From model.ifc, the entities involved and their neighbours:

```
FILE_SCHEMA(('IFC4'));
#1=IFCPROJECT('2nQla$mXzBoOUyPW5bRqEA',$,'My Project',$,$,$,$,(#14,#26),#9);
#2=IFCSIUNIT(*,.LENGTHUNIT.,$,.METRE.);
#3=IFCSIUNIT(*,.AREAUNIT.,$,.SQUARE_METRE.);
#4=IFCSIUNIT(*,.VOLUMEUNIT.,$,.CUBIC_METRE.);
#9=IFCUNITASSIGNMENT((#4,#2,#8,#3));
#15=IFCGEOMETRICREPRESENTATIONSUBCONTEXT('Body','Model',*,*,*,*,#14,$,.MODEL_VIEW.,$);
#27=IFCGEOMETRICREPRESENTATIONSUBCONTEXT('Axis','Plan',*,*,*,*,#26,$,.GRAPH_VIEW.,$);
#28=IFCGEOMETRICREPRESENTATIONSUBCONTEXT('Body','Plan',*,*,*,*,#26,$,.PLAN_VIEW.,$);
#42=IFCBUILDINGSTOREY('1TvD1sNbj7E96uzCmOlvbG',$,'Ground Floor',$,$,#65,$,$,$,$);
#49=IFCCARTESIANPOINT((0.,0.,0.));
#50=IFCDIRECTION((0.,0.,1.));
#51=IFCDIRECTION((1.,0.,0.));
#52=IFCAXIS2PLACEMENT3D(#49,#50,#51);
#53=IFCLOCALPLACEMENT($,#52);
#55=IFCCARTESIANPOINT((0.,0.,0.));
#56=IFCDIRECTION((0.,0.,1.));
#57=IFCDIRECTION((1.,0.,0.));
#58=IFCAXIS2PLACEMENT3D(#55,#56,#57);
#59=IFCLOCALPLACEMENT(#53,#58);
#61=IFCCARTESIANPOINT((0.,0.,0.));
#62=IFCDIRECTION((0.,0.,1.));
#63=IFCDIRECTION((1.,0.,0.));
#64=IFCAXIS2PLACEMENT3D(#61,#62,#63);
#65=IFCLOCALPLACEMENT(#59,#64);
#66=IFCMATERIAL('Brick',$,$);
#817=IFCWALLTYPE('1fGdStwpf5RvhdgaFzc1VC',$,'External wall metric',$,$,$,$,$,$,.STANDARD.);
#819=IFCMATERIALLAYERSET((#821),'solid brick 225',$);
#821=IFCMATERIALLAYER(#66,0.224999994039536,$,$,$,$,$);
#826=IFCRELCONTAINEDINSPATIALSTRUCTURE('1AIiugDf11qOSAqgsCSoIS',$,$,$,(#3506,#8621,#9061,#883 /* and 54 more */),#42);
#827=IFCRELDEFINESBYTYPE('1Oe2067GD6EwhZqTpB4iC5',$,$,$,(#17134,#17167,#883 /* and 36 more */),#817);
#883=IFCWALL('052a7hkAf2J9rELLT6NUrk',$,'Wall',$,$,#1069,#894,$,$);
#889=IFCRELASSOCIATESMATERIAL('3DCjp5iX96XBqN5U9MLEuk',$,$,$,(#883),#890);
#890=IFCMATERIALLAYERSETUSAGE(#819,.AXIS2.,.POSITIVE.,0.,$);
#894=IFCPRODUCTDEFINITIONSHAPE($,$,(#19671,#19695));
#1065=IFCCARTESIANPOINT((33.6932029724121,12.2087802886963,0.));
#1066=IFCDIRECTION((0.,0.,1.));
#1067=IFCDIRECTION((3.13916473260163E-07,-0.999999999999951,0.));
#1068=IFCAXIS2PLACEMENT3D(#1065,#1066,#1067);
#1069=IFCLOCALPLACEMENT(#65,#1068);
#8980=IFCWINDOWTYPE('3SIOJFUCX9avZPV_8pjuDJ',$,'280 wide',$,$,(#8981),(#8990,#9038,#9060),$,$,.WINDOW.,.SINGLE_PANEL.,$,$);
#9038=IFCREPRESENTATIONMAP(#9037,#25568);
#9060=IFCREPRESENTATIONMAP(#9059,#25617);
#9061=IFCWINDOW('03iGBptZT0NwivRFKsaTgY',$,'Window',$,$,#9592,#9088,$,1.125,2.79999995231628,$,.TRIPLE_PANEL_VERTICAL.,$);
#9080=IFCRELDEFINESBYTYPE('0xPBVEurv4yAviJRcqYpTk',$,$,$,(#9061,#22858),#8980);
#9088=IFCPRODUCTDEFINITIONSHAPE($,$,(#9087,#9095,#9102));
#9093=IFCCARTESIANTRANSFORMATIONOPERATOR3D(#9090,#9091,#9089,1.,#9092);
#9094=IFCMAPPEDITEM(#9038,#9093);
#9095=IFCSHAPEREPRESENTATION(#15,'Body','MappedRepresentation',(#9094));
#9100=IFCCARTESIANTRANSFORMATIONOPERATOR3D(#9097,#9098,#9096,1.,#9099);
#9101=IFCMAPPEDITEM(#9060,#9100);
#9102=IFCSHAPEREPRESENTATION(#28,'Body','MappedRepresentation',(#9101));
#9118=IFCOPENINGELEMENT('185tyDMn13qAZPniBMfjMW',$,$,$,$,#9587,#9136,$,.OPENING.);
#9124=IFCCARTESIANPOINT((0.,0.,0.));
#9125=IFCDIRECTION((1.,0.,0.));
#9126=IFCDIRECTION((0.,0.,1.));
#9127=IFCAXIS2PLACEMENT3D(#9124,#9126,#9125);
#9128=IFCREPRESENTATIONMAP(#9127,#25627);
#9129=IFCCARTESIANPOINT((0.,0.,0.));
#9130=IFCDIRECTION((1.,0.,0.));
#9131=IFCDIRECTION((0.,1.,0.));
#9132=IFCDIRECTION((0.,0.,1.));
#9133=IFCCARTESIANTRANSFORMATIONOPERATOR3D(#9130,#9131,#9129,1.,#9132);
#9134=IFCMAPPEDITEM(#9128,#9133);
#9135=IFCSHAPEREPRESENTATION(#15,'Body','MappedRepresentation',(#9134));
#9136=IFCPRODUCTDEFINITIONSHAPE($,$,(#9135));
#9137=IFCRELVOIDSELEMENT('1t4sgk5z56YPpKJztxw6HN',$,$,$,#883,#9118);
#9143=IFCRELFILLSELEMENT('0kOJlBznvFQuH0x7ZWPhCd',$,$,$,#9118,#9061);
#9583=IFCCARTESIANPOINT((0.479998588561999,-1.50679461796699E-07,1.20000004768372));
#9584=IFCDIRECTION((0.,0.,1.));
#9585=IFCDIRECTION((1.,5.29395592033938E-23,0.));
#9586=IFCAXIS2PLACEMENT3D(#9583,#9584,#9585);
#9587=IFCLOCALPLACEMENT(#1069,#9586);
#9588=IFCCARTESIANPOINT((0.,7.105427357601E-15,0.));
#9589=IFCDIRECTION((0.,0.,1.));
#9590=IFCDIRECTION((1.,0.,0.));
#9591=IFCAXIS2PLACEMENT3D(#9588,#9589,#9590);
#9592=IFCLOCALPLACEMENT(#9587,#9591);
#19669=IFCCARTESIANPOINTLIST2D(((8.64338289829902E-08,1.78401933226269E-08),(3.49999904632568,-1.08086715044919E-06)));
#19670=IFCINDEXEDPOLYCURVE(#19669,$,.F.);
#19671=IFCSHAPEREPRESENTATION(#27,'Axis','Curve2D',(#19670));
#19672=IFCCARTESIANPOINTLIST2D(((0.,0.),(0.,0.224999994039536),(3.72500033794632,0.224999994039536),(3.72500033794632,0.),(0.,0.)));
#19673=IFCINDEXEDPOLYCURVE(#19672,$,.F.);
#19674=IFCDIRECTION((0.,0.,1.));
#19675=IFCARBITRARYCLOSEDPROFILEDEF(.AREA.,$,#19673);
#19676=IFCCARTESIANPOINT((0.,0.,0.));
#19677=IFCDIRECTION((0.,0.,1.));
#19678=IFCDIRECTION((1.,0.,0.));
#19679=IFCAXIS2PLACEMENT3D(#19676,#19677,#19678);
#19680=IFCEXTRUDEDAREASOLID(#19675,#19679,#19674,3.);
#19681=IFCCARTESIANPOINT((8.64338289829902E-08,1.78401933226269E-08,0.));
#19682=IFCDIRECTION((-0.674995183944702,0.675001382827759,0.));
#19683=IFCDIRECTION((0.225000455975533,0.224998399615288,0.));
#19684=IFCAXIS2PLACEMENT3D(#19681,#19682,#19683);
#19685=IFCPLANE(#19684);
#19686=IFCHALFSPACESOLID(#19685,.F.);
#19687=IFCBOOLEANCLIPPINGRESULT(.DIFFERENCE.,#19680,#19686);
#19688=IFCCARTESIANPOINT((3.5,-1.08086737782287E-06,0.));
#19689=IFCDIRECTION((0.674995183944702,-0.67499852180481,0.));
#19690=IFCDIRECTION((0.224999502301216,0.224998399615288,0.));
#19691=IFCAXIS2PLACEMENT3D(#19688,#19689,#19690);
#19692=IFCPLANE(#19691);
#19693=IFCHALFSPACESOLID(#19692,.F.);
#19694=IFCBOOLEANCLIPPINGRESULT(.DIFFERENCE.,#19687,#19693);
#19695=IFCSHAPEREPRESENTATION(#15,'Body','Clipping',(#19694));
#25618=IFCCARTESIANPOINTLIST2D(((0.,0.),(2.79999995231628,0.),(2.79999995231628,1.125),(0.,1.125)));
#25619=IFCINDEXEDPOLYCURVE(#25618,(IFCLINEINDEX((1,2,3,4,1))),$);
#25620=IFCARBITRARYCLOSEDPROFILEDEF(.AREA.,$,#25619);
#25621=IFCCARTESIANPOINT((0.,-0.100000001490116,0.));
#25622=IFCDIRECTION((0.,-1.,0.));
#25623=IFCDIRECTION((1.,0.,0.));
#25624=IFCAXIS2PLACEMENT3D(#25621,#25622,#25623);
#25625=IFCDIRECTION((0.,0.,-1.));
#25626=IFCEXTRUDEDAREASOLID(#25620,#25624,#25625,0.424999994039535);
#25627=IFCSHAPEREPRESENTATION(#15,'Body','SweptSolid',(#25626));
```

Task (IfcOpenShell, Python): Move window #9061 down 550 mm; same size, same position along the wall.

```python
import numpy as np
import ifcopenshell
import ifcopenshell.api.geometry
import ifcopenshell.util.placement
import ifcopenshell.util.unit

model = ifcopenshell.open("model.ifc")
unit_scale = ifcopenshell.util.unit.calculate_unit_scale(model)

window = model.by_guid("03iGBptZT0NwivRFKsaTgY")
opening = window.FillsVoids[0].RelatingOpeningElement
dz = -0.55 / unit_scale

shift = np.array([0.0, 0.0, dz])
# The window is placed relative to its opening, so it follows when the opening moves.
matrix = ifcopenshell.util.placement.get_local_placement(opening.ObjectPlacement)
matrix[:3, 3] += shift
ifcopenshell.api.geometry.edit_object_placement(
    model, product=opening, matrix=matrix, is_si=False, should_transform_children=True
)

print(f"moved by {dz * unit_scale:+.3f} m")

model.write("model_edited.ifc")
```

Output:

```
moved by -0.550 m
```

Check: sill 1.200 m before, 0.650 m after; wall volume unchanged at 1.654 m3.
